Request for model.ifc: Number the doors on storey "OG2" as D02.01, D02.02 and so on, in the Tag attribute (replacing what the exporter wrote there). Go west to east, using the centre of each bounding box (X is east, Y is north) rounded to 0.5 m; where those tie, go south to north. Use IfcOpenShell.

First a look at what the model holds.

```python
import ifcopenshell
import ifcopenshell.util.element
import ifcopenshell.util.placement

model = ifcopenshell.open("model.ifc")
print(model.schema)
storey = next(s for s in model.by_type("IfcBuildingStorey") if s.Name == "OG2")
doors = [e for e in ifcopenshell.util.element.get_decomposition(storey) if e.is_a("IfcDoor")]
for e in sorted(doors, key=lambda e: e.id()):
    origin = ifcopenshell.util.placement.get_local_placement(e.ObjectPlacement)[:3, 3]
    print(e.id(), e.Tag, e.Name, origin.round(2) + 0.0, sep=" | ")
```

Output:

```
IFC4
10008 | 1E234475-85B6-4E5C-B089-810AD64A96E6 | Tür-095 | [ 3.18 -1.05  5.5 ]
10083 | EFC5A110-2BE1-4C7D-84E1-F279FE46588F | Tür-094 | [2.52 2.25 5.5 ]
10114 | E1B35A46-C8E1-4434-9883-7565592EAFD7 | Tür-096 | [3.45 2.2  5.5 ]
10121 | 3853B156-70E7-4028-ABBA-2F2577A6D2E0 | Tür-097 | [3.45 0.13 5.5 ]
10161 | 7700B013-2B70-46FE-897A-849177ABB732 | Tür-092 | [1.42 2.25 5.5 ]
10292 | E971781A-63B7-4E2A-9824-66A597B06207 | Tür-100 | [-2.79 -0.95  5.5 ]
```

```python
import ifcopenshell
import ifcopenshell.geom
import ifcopenshell.util.element
import ifcopenshell.util.shape

model = ifcopenshell.open("model.ifc")
settings = ifcopenshell.geom.settings()
settings.set("use-world-coords", True)


def centre(element):
    shape = ifcopenshell.geom.create_shape(settings, element)
    return ifcopenshell.util.shape.get_bbox_centroid(shape.geometry)


storey = next(s for s in model.by_type("IfcBuildingStorey") if s.Name == "OG2")
doors = [e for e in ifcopenshell.util.element.get_decomposition(storey) if e.is_a("IfcDoor")]

# Insertion points can sit at a corner or the storey origin, so sort by the geometry (in metres).
centres = {e: centre(e) for e in doors}
doors.sort(key=lambda e: (round(centres[e][0] / 0.5), centres[e][1]))

for i, e in enumerate(doors, start=1):
    number = f"D02.{i:02d}"
    e.Tag = number
    print(e.id(), number)

model.write("model_v2.ifc")
```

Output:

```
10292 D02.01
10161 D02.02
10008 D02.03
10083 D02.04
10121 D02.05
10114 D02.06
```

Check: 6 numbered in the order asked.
